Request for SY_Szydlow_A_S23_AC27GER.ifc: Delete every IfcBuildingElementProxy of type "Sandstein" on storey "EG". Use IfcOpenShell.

First a look at what the model holds.

```python
import ifcopenshell
import ifcopenshell.util.element

model = ifcopenshell.open("SY_Szydlow_A_S23_AC27GER.ifc")
print(model.schema)
storey = next(s for s in model.by_type("IfcBuildingStorey") if s.Name == "EG")
proxies = [e for e in ifcopenshell.util.element.get_decomposition(storey) if e.is_a("IfcBuildingElementProxy")]
seen = {}
for e in proxies:
    element_type = ifcopenshell.util.element.get_type(e)
    name = element_type.Name if element_type not in (None, e) else None
    seen[name] = seen.get(name, 0) + 1
for name, count in sorted(seen.items(), key=str):
    print(count, "x", name)
```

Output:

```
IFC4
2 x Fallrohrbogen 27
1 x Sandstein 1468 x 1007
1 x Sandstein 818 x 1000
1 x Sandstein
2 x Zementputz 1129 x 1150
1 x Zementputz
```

```python
import ifcopenshell
import ifcopenshell.api.root
import ifcopenshell.util.element

model = ifcopenshell.open("SY_Szydlow_A_S23_AC27GER.ifc")

storey = next(s for s in model.by_type("IfcBuildingStorey") if s.Name == "EG")
proxies = [e for e in ifcopenshell.util.element.get_decomposition(storey) if e.is_a("IfcBuildingElementProxy")]
targets = [e for e in proxies if (t := ifcopenshell.util.element.get_type(e)) not in (None, e) and t.Name == "Sandstein"]

for e in targets:
    ifcopenshell.api.root.remove_product(model, product=e)
print(len(targets), "removed")

model.write("SY_Szydlow_A_S23_AC27GER-out.ifc")
```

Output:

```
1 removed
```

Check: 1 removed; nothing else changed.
